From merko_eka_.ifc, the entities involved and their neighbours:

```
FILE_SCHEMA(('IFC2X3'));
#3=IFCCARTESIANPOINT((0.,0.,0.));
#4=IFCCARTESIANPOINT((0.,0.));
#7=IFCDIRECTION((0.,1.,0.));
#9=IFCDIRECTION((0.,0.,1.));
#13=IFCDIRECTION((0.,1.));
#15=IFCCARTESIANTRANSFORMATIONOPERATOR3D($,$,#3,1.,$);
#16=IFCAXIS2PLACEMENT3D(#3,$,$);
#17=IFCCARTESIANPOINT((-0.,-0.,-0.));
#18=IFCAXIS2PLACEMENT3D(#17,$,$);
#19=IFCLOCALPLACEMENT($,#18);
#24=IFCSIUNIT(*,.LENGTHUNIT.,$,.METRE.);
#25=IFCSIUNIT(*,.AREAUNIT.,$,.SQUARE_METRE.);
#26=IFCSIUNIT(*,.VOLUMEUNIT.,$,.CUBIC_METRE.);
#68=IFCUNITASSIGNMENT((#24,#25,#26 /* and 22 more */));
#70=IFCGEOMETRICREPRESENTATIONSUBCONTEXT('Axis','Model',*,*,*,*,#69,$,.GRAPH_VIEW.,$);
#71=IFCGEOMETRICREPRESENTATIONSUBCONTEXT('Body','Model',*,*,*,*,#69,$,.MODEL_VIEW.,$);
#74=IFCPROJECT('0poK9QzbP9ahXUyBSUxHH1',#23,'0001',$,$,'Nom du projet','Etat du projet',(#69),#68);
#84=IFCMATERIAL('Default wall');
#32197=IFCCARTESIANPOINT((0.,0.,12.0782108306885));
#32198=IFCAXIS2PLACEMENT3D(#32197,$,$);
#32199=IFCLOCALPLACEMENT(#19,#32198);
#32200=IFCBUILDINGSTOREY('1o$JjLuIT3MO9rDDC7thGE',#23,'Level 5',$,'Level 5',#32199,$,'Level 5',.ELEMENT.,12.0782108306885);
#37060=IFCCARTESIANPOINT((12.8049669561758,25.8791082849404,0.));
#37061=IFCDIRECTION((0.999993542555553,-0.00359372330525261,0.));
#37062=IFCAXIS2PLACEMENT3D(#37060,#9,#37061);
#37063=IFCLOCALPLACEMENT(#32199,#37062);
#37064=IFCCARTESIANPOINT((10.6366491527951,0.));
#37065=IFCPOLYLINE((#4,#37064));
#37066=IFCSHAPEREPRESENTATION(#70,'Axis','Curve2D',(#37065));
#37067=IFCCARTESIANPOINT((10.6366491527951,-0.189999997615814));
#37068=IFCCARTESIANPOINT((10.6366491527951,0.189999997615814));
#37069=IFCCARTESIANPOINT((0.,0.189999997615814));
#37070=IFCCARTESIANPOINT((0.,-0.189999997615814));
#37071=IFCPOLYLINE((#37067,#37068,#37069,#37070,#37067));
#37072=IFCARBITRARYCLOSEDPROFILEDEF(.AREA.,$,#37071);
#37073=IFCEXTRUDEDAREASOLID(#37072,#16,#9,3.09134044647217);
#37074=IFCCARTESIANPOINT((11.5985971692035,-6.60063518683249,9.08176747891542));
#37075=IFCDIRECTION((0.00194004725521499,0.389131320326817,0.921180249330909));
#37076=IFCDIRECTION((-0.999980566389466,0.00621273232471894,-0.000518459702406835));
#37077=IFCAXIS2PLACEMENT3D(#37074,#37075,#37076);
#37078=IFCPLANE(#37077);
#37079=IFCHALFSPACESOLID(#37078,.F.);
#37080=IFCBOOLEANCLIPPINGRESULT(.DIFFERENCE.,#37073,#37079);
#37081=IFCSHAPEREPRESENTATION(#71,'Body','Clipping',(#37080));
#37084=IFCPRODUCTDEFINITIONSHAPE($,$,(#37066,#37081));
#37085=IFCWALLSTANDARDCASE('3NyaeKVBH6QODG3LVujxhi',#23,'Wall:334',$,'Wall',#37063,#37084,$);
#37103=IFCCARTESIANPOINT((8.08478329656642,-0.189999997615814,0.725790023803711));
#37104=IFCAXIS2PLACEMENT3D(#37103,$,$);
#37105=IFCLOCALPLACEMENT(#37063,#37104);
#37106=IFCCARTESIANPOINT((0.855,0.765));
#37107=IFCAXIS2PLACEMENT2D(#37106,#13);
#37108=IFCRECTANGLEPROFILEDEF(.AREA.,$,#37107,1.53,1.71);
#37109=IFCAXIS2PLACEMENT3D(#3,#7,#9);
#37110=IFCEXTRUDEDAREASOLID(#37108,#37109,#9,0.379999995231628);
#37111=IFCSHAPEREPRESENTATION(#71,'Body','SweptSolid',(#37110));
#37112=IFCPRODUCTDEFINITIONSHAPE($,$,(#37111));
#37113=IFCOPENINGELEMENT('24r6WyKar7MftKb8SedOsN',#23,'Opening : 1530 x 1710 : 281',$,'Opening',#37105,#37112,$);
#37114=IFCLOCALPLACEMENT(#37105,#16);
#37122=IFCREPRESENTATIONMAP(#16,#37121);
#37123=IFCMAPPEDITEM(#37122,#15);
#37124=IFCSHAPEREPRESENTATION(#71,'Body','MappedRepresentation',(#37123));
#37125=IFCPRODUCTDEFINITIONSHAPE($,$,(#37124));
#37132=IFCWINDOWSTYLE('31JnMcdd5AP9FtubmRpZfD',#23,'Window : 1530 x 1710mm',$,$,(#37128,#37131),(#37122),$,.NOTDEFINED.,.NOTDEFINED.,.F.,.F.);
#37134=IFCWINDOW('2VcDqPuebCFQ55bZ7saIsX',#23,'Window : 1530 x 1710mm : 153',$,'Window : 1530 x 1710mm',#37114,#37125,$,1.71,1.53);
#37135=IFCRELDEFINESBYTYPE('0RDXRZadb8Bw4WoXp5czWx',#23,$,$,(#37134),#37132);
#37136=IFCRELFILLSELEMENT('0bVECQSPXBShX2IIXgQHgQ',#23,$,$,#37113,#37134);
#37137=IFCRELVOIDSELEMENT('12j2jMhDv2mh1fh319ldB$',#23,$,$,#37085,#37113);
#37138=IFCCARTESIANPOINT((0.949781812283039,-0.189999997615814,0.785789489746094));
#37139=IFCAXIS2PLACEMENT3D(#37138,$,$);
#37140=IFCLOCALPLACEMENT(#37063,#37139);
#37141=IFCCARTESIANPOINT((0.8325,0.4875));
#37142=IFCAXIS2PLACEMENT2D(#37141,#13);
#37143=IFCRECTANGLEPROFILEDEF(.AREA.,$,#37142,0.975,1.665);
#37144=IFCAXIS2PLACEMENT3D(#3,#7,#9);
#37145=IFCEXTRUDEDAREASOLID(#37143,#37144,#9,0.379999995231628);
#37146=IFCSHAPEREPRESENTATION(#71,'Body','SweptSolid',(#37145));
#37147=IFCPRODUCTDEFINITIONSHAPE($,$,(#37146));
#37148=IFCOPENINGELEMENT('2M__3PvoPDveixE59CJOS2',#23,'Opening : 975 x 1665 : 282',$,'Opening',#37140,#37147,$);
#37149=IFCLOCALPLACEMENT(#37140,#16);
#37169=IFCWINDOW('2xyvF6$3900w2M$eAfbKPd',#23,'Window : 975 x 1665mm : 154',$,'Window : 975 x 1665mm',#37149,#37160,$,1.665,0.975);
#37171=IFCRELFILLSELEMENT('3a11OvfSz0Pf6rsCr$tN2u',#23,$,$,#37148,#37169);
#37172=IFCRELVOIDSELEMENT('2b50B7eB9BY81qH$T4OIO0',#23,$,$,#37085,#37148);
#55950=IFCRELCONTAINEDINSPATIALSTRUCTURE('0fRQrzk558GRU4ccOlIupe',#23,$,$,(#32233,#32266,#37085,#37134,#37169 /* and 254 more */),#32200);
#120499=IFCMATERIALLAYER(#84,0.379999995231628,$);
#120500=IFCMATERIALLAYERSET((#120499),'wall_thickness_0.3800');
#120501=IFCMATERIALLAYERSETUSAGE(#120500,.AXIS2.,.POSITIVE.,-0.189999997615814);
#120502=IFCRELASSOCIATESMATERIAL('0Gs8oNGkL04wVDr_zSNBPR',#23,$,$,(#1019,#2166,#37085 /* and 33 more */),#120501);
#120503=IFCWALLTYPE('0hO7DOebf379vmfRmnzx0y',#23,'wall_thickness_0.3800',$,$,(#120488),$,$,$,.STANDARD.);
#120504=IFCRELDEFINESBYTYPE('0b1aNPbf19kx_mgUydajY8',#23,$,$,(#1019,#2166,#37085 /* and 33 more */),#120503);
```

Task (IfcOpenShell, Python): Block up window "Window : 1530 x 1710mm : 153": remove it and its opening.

```python
import ifcopenshell
import ifcopenshell.api.feature
import ifcopenshell.api.root
import ifcopenshell.geom
import ifcopenshell.util.shape

model = ifcopenshell.open("merko_eka_.ifc")
settings = ifcopenshell.geom.settings()


def volume(element):
    """Net volume in cubic metres, openings subtracted."""
    shape = ifcopenshell.geom.create_shape(settings, element)
    return ifcopenshell.util.shape.get_volume(shape.geometry)


window = model.by_id(37134)
opening = window.FillsVoids[0].RelatingOpeningElement
wall = opening.VoidsElements[0].RelatingBuildingElement
before = volume(wall)

ifcopenshell.api.root.remove_product(model, product=window)
ifcopenshell.api.feature.remove_feature(model, feature=opening)

after = volume(wall)

print(f"wall volume {before:.3f} -> {after:.3f} m3")

model.write("merko_eka_-out.ifc")
```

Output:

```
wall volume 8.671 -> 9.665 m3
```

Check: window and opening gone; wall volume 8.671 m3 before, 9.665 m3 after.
